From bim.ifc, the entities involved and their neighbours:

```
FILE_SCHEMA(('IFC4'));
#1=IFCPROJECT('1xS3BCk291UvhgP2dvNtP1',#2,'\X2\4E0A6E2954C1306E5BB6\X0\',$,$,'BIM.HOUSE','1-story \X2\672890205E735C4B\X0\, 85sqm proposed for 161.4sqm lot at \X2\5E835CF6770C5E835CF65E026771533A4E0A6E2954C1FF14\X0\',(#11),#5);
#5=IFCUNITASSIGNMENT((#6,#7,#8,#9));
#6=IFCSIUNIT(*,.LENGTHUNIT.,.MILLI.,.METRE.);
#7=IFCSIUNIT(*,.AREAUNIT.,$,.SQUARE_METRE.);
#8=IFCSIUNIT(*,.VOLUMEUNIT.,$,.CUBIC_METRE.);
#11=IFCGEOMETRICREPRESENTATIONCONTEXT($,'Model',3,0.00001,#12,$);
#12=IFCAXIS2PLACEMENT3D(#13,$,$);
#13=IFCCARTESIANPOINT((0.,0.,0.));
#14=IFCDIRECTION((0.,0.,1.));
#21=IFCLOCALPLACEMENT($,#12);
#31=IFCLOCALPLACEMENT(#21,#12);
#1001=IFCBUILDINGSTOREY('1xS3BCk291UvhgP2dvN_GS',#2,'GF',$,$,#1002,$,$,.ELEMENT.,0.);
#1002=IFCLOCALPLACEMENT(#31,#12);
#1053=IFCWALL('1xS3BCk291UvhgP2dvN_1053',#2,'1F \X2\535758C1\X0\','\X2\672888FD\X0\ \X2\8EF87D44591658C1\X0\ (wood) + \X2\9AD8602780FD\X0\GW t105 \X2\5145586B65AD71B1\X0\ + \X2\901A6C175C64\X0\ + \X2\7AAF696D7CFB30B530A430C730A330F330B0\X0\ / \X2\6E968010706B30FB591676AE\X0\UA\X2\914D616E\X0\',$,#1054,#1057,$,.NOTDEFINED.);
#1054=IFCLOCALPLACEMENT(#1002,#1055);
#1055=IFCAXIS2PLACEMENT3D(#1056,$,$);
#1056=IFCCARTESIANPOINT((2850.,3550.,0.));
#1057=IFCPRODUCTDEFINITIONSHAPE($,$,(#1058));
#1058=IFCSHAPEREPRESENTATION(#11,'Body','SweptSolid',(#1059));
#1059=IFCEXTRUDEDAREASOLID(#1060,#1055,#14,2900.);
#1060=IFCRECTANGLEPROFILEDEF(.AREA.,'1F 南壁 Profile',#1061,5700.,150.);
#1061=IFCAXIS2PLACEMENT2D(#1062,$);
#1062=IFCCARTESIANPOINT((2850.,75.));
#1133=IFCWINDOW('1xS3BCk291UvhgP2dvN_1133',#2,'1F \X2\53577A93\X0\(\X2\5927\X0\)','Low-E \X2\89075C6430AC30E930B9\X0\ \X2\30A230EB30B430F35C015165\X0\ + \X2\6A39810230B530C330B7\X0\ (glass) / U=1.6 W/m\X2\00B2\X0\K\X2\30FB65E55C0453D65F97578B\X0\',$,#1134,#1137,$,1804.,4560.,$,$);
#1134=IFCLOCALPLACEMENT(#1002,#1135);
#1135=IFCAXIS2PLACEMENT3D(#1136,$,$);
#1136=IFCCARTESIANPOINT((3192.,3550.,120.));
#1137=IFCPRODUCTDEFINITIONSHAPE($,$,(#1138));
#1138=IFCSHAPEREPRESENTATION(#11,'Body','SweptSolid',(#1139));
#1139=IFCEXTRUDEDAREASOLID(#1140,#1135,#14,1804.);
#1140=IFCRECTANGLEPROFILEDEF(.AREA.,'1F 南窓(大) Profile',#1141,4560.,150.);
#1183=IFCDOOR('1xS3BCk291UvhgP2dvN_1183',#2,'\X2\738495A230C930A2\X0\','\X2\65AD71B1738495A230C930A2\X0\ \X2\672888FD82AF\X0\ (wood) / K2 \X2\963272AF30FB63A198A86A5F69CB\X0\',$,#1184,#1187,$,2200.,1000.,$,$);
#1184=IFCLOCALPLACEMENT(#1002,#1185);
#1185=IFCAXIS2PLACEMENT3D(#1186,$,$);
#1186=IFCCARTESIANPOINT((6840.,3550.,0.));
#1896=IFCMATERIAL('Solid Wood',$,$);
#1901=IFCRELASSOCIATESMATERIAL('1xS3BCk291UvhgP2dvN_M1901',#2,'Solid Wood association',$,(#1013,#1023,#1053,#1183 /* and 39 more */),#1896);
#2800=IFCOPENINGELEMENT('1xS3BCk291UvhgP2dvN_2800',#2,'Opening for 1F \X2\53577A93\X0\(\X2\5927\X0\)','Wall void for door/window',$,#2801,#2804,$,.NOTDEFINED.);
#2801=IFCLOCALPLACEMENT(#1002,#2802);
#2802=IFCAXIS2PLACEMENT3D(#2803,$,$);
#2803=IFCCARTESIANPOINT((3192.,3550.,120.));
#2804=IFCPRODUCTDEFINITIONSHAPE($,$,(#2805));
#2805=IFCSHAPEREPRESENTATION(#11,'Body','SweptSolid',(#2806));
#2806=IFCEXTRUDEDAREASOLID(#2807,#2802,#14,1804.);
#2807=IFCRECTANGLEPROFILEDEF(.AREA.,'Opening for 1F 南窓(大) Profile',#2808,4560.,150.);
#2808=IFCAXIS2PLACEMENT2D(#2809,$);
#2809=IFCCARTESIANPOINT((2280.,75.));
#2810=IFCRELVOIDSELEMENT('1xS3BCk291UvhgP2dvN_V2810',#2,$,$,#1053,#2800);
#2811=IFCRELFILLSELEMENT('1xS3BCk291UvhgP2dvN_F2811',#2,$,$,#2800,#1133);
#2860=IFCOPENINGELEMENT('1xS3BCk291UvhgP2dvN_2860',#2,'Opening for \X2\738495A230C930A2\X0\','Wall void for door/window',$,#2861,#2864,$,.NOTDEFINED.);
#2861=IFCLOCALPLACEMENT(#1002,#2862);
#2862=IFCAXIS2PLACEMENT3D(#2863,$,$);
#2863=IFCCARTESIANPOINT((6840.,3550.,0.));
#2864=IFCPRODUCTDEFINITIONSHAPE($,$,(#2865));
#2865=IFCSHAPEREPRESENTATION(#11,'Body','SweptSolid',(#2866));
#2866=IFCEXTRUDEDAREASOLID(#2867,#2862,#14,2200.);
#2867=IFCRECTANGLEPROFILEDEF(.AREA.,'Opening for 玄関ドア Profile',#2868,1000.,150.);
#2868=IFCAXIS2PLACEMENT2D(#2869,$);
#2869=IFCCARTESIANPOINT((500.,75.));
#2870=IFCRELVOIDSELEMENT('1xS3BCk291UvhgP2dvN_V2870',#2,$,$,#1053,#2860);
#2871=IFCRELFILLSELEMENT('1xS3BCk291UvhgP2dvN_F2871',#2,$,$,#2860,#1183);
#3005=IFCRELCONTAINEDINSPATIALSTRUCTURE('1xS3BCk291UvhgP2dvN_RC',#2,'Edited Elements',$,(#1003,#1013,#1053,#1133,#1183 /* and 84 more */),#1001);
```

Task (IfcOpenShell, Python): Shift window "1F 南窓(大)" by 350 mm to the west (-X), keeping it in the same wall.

```python
import ifcopenshell
import ifcopenshell.api.geometry
import ifcopenshell.util.placement

model = ifcopenshell.open("bim.ifc")

window = model.by_guid("1xS3BCk291UvhgP2dvN_1133")
opening = window.FillsVoids[0].RelatingOpeningElement
wall = opening.VoidsElements[0].RelatingBuildingElement

wall_matrix = ifcopenshell.util.placement.get_local_placement(wall.ObjectPlacement)
shift = wall_matrix[:3, 0] * -350.0
before = ifcopenshell.util.placement.get_local_placement(window.ObjectPlacement)[:3, 3].copy()

# The window is not placed relative to its opening, so move both.
for product in (opening, window):
    matrix = ifcopenshell.util.placement.get_local_placement(product.ObjectPlacement)
    matrix[:3, 3] += shift
    ifcopenshell.api.geometry.edit_object_placement(model, product=product, matrix=matrix, is_si=False)

after = ifcopenshell.util.placement.get_local_placement(window.ObjectPlacement)[:3, 3]
print("window moved by", (after - before).round(3) + 0.0)

model.write("bim_rev.ifc")
```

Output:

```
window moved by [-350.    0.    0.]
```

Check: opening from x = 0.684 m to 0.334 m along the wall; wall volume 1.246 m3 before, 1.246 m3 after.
